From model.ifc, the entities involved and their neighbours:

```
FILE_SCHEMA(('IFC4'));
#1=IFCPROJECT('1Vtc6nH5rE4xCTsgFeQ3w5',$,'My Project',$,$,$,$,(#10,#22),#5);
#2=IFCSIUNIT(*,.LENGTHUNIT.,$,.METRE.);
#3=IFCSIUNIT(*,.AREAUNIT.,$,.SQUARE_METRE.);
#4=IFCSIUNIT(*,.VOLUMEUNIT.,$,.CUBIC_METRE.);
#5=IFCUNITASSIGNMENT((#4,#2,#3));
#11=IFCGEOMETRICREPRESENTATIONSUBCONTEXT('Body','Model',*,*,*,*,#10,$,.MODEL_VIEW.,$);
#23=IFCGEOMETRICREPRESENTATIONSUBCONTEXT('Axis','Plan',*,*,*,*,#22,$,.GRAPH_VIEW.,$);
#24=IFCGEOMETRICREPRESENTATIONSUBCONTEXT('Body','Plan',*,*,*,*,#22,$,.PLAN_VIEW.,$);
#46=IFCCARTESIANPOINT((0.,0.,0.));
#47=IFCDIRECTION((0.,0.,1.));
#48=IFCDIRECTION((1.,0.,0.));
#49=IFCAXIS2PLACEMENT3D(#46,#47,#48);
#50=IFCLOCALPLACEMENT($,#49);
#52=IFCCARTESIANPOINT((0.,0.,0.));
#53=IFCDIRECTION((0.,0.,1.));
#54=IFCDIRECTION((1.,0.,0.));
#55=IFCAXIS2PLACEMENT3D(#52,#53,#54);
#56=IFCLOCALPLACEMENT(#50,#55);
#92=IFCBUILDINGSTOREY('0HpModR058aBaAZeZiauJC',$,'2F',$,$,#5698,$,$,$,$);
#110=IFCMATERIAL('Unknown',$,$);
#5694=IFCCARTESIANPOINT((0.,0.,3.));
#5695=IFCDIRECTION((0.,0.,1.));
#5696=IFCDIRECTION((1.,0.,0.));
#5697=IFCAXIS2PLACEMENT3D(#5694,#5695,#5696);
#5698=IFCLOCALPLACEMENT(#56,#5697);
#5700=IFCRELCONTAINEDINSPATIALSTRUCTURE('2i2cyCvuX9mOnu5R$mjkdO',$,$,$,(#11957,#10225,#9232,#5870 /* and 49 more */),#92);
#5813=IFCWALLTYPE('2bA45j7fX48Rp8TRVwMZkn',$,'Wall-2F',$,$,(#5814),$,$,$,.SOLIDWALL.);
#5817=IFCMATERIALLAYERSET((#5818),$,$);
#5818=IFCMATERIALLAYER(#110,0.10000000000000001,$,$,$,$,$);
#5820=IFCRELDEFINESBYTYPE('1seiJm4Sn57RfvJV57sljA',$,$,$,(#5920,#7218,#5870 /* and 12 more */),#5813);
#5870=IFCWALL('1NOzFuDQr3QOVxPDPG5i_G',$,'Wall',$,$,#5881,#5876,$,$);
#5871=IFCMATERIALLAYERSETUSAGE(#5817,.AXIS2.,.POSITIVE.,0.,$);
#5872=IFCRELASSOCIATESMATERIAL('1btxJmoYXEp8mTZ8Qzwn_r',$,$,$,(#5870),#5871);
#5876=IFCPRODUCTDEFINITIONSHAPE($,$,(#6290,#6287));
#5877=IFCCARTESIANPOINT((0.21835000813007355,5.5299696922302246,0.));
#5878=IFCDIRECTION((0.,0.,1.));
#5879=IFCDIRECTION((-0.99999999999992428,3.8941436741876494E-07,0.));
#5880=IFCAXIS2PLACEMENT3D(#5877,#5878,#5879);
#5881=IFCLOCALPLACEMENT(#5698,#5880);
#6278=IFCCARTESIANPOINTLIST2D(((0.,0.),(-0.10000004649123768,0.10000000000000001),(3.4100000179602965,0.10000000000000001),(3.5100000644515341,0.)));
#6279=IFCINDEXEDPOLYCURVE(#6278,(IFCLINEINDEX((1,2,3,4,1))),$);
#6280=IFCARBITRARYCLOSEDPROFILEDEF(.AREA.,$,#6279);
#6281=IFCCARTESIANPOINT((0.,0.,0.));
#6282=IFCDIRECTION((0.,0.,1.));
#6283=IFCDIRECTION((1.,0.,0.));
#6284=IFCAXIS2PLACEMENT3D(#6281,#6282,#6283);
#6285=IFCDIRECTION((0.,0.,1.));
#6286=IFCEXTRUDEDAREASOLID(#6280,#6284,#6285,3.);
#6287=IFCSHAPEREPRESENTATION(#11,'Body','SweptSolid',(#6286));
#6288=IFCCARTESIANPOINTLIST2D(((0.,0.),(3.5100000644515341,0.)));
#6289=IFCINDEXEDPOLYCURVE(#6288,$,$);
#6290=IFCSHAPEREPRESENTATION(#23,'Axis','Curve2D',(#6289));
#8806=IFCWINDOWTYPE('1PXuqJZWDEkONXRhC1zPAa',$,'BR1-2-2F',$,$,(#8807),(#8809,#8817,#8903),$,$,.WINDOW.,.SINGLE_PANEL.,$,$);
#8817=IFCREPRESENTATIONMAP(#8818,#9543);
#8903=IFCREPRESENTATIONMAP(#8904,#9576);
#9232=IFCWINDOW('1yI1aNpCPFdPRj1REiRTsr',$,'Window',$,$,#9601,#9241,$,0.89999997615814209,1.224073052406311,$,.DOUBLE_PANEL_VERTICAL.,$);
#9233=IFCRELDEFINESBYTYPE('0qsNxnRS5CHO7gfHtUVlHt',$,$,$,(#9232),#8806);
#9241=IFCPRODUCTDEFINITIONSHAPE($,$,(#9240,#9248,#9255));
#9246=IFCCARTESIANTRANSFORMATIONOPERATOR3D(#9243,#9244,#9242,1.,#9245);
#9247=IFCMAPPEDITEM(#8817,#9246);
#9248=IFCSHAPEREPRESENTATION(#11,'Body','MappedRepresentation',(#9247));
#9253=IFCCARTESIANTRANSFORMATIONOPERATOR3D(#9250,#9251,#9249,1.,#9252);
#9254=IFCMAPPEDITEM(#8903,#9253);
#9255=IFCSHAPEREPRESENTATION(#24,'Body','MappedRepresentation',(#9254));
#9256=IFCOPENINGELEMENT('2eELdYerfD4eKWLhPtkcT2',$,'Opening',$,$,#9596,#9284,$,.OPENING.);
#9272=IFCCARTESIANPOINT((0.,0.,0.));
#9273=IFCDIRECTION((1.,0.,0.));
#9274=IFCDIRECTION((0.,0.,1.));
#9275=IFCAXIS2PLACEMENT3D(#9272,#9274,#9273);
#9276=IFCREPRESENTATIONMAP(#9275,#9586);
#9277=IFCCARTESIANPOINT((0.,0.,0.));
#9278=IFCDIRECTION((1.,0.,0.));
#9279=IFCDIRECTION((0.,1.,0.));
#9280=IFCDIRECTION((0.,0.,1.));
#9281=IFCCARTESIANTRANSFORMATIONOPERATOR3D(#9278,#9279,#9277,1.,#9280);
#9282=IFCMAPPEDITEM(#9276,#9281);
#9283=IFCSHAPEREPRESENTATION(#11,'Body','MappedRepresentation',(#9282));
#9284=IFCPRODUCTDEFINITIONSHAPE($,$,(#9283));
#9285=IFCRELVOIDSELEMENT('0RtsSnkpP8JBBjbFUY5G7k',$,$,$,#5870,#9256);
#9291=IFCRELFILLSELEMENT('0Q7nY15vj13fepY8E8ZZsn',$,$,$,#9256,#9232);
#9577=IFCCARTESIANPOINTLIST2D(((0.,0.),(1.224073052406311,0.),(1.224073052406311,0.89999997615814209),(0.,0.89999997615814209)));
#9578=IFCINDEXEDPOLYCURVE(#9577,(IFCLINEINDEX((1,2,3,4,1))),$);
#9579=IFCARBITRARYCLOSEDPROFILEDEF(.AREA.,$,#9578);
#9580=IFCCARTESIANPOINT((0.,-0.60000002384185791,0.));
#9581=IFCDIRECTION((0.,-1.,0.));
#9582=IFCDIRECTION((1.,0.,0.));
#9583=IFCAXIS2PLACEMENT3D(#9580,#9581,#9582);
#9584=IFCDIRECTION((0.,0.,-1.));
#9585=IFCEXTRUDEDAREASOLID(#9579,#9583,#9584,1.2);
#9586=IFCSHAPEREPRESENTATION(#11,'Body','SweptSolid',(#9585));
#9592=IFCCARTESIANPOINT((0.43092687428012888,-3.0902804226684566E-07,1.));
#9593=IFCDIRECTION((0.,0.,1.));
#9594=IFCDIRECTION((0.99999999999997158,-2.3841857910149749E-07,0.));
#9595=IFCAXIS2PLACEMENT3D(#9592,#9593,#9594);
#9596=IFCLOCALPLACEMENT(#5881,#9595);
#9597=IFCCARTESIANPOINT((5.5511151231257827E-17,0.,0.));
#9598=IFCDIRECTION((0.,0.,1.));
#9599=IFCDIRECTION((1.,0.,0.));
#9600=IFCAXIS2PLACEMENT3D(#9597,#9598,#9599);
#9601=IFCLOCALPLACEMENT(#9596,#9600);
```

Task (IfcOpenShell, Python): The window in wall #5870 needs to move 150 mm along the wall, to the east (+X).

```python
import ifcopenshell
import ifcopenshell.api.geometry
import ifcopenshell.util.placement

model = ifcopenshell.open("model.ifc")

window = model.by_id(9232)
opening = window.FillsVoids[0].RelatingOpeningElement
wall = opening.VoidsElements[0].RelatingBuildingElement

wall_matrix = ifcopenshell.util.placement.get_local_placement(wall.ObjectPlacement)
shift = wall_matrix[:3, 0] * -0.15
before = ifcopenshell.util.placement.get_local_placement(window.ObjectPlacement)[:3, 3].copy()

# The window is placed relative to its opening, so it follows when the opening moves.
matrix = ifcopenshell.util.placement.get_local_placement(opening.ObjectPlacement)
matrix[:3, 3] += shift
ifcopenshell.api.geometry.edit_object_placement(
    model, product=opening, matrix=matrix, is_si=False, should_transform_children=True
)

after = ifcopenshell.util.placement.get_local_placement(window.ObjectPlacement)[:3, 3]
print("window moved by", (after - before).round(3) + 0.0)

model.write("model_edited.ifc")
```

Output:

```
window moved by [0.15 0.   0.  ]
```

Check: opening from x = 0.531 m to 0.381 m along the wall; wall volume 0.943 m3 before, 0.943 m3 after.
